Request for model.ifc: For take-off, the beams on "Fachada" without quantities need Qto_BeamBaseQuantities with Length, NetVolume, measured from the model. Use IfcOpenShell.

First a look at what the model holds.

```python
import ifcopenshell
import ifcopenshell.util.element
import ifcopenshell.util.unit

model = ifcopenshell.open("model.ifc")
print(model.schema)
for unit_type in ("LENGTHUNIT", "AREAUNIT", "VOLUMEUNIT"):
    print(unit_type, ifcopenshell.util.unit.calculate_unit_scale(model, unit_type))
storey = next(s for s in model.by_type("IfcBuildingStorey") if s.Name == "Fachada")
beams = [e for e in ifcopenshell.util.element.get_decomposition(storey) if e.is_a("IfcBeam")]
for e in sorted(beams, key=lambda e: e.id()):
    print(e.id(), e.is_a(), e.Name, list(ifcopenshell.util.element.get_psets(e, qtos_only=True)), sep=" | ")
```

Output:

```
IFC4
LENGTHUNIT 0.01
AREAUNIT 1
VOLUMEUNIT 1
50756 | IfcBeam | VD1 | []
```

```python
import ifcopenshell
import ifcopenshell.api.pset
import ifcopenshell.geom
import ifcopenshell.util.element
import ifcopenshell.util.shape
import ifcopenshell.util.unit

model = ifcopenshell.open("model.ifc")
unit_scale = ifcopenshell.util.unit.calculate_unit_scale(model)
volume_scale = ifcopenshell.util.unit.calculate_unit_scale(model, "VOLUMEUNIT")
settings = ifcopenshell.geom.settings()

storey = next(s for s in model.by_type("IfcBuildingStorey") if s.Name == "Fachada")
beams = [e for e in ifcopenshell.util.element.get_decomposition(storey) if e.is_a("IfcBeam")]

for e in sorted(beams, key=lambda e: e.id()):
    if ifcopenshell.util.element.get_psets(e, qtos_only=True, should_inherit=False):
        continue
    # Geometry comes back in metres, in the element's own axes.
    shape = ifcopenshell.geom.create_shape(settings, e)
    values = {
        "Length": ifcopenshell.util.shape.get_max_xyz(shape.geometry) / unit_scale,
        "NetVolume": ifcopenshell.util.shape.get_volume(shape.geometry) / volume_scale,
    }
    qto = ifcopenshell.api.pset.add_qto(model, product=e, name="Qto_BeamBaseQuantities")
    ifcopenshell.api.pset.edit_qto(model, qto=qto, properties=values)
    print(e.id(), {k: round(v, 3) for k, v in values.items()})

model.write("model_edited.ifc")
```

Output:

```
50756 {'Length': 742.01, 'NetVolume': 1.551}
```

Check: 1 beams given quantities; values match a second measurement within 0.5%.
